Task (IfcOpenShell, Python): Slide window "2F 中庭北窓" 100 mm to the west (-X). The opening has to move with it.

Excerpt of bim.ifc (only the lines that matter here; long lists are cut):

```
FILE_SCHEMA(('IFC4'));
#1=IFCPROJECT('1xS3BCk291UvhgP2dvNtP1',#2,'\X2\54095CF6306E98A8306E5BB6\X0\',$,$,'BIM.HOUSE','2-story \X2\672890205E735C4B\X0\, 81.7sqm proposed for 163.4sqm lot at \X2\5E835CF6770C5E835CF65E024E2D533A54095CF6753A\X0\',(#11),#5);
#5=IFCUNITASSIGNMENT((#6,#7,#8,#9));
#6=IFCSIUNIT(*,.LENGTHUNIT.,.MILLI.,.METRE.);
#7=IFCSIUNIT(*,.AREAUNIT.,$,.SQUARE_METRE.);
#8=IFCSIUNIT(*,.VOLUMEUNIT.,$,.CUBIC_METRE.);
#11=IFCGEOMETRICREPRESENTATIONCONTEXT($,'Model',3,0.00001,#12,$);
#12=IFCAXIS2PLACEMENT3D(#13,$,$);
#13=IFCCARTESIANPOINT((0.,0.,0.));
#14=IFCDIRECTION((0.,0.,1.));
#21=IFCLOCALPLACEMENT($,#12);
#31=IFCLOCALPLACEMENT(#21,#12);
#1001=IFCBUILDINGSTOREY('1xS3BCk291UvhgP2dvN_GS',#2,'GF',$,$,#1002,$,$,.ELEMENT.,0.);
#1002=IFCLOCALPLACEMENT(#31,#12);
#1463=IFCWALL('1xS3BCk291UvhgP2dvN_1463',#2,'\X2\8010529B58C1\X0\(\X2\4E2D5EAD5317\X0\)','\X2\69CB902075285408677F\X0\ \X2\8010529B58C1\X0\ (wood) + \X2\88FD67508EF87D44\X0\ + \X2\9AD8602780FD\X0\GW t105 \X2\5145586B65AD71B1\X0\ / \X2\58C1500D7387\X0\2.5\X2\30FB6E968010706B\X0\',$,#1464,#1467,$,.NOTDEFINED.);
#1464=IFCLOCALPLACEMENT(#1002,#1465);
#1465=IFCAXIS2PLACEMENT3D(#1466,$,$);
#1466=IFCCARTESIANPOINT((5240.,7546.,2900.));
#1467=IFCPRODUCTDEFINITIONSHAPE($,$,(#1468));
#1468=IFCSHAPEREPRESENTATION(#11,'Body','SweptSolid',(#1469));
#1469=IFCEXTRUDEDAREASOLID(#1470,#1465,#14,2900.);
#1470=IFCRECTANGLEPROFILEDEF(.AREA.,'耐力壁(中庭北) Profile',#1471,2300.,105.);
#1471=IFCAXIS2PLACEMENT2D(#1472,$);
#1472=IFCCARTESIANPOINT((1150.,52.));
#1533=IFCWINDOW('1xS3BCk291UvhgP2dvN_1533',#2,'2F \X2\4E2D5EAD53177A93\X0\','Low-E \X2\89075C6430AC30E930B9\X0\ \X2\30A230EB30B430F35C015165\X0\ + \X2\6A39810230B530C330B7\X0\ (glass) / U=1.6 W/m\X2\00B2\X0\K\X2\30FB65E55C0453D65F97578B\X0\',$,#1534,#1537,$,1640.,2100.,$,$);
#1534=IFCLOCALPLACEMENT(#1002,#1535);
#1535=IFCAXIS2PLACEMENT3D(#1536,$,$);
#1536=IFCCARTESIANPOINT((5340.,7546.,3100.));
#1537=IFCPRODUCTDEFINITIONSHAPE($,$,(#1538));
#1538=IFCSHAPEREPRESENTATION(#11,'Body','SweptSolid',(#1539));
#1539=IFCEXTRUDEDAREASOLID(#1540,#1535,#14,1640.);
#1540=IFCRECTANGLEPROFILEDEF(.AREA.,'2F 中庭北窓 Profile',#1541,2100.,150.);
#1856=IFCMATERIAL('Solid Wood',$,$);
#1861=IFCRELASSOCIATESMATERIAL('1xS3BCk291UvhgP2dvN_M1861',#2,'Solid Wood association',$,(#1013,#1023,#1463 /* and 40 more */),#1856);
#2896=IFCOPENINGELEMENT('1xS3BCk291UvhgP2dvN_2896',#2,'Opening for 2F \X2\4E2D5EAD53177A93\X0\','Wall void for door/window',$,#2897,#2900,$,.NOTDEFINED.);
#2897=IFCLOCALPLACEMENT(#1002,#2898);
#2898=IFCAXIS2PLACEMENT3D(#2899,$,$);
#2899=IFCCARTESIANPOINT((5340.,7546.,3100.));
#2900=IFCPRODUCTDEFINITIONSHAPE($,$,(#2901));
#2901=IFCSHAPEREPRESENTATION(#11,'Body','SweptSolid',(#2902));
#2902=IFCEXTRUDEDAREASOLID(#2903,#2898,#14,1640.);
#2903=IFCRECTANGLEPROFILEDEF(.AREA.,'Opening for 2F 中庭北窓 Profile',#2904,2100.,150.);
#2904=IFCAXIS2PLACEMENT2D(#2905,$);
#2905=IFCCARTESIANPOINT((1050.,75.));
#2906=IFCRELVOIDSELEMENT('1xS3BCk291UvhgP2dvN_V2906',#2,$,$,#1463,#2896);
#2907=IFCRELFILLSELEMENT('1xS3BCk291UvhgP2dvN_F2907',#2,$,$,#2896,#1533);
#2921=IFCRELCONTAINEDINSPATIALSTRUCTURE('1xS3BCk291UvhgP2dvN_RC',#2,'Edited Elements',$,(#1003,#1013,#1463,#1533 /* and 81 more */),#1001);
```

```python
import ifcopenshell
import ifcopenshell.api.geometry
import ifcopenshell.util.placement

model = ifcopenshell.open("bim.ifc")

window = model.by_id(1533)
opening = window.FillsVoids[0].RelatingOpeningElement
wall = opening.VoidsElements[0].RelatingBuildingElement

wall_matrix = ifcopenshell.util.placement.get_local_placement(wall.ObjectPlacement)
shift = wall_matrix[:3, 0] * -100.0
before = ifcopenshell.util.placement.get_local_placement(window.ObjectPlacement)[:3, 3].copy()

# The window is not placed relative to its opening, so move both.
for product in (opening, window):
    matrix = ifcopenshell.util.placement.get_local_placement(product.ObjectPlacement)
    matrix[:3, 3] += shift
    ifcopenshell.api.geometry.edit_object_placement(model, product=product, matrix=matrix, is_si=False)

after = ifcopenshell.util.placement.get_local_placement(window.ObjectPlacement)[:3, 3]
print("window moved by", (after - before).round(3) + 0.0)

model.write("bim_v2.ifc")
```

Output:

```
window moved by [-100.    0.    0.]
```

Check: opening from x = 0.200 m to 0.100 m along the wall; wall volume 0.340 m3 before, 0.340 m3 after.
